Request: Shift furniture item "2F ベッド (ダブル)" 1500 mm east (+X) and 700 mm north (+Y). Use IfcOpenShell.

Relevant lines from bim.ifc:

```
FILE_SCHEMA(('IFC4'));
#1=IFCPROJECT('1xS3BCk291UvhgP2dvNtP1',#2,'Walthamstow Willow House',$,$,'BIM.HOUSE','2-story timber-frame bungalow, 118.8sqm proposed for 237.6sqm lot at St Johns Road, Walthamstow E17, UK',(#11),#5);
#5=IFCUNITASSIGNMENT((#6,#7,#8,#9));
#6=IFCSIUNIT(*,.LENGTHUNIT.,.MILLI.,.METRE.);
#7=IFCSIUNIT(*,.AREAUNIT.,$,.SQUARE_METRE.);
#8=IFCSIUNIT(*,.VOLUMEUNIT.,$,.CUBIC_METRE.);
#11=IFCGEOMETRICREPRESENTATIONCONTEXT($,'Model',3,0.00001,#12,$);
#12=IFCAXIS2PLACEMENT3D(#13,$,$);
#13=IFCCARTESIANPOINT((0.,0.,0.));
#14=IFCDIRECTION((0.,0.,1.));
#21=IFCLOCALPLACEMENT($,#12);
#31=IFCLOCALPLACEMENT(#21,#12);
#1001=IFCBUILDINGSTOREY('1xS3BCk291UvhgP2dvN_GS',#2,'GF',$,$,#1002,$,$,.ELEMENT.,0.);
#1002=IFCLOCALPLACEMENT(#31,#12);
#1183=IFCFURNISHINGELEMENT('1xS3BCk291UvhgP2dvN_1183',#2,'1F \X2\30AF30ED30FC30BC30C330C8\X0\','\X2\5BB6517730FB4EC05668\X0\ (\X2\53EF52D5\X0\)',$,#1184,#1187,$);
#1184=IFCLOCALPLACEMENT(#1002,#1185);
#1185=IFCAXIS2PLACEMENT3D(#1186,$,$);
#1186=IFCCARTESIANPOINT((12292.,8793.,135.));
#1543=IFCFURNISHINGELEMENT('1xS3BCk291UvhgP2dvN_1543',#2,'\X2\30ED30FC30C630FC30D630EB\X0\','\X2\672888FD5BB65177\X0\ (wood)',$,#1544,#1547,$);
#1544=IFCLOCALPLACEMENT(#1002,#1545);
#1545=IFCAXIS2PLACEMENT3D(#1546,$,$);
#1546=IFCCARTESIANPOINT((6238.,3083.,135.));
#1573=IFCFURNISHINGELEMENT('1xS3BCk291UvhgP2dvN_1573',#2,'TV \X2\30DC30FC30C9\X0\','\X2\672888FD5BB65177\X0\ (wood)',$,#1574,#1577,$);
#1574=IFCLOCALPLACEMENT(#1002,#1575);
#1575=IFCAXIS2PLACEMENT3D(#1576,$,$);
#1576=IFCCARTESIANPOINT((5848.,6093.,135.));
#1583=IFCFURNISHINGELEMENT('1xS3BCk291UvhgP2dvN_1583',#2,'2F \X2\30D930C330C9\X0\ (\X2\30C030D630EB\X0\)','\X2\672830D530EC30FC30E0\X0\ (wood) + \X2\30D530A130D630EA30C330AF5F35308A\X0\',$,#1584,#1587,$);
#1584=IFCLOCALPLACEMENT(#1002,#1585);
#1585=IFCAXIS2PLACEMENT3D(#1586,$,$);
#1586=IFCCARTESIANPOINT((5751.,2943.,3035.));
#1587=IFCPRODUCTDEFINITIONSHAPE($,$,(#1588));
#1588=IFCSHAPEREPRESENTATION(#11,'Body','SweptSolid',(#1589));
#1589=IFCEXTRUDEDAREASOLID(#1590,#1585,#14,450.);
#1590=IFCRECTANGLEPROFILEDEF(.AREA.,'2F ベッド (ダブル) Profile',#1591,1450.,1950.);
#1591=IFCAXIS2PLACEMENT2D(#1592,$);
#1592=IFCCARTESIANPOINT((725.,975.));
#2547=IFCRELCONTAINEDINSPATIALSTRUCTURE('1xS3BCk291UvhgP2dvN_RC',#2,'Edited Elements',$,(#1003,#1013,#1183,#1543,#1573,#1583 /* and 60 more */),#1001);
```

```python
import ifcopenshell
import ifcopenshell.api.geometry
import ifcopenshell.util.placement

model = ifcopenshell.open("bim.ifc")

item = model.by_id(1583)
matrix = ifcopenshell.util.placement.get_local_placement(item.ObjectPlacement)
matrix[0, 3] += 1500.0
matrix[1, 3] += 700.0
ifcopenshell.api.geometry.edit_object_placement(model, product=item, matrix=matrix, is_si=False)

print(ifcopenshell.util.placement.get_local_placement(item.ObjectPlacement).round(3) + 0.0)

model.write("bim_rev.ifc")
```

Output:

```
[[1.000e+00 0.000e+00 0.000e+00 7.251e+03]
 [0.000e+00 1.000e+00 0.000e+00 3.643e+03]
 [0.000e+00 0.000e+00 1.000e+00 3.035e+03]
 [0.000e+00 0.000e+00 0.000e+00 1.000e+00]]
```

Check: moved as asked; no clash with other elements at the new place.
